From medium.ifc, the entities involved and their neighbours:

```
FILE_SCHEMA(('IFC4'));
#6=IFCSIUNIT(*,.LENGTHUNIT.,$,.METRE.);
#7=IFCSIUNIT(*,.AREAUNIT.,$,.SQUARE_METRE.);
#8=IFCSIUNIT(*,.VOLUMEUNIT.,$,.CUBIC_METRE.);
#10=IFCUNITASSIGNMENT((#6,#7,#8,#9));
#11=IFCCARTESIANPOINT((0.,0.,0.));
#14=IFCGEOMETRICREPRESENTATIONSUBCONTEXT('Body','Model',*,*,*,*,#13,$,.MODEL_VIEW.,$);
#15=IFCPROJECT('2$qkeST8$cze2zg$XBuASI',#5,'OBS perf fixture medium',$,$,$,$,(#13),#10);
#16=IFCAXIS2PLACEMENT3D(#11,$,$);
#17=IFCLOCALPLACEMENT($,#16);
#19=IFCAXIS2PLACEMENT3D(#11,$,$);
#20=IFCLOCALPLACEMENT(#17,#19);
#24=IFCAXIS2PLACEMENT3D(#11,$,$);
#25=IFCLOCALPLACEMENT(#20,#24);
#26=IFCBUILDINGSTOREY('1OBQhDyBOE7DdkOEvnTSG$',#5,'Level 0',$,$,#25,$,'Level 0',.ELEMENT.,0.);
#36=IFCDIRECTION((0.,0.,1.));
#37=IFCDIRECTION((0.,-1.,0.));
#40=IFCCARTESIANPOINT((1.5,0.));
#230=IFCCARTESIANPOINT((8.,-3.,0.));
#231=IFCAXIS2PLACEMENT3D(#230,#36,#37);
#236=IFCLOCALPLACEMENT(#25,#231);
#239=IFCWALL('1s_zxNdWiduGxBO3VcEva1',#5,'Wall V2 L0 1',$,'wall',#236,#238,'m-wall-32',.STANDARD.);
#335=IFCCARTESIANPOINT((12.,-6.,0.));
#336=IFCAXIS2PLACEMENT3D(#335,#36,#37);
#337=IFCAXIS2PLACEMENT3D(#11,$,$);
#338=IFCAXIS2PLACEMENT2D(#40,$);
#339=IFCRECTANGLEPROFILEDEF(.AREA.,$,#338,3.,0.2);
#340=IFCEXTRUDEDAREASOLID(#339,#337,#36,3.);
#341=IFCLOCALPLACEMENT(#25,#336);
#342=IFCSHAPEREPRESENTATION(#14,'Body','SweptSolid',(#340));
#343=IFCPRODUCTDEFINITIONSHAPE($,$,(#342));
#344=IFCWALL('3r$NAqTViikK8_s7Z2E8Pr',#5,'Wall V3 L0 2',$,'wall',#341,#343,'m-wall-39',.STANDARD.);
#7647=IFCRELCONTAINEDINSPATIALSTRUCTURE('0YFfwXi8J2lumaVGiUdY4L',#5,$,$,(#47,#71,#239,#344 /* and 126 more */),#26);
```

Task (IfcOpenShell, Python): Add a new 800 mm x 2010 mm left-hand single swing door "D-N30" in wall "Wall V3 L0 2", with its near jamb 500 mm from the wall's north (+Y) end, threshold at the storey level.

```python
import numpy as np
import ifcopenshell
import ifcopenshell.api.feature
import ifcopenshell.api.geometry
import ifcopenshell.api.root
import ifcopenshell.api.spatial
import ifcopenshell.geom
import ifcopenshell.util.element
import ifcopenshell.util.placement
import ifcopenshell.util.representation
import ifcopenshell.util.shape
import ifcopenshell.util.unit

model = ifcopenshell.open("medium.ifc")
unit_scale = ifcopenshell.util.unit.calculate_unit_scale(model)
settings = ifcopenshell.geom.settings()


def volume(element):
    """Net volume in cubic metres, openings subtracted."""
    shape = ifcopenshell.geom.create_shape(settings, element)
    return ifcopenshell.util.shape.get_volume(shape.geometry)


wall = model.by_guid("3r$NAqTViikK8_s7Z2E8Pr")
storey = ifcopenshell.util.element.get_container(wall, ifc_class="IfcBuildingStorey")
context = ifcopenshell.util.representation.get_context(model, "Model", "Body", "MODEL_VIEW")
before = volume(wall)

width, height, from_end, sill = 0.8, 2.01, 0.5, 0.0  # metres

# The wall runs along its own X axis, and the end named is its -X end.
wall_shape = ifcopenshell.geom.create_shape(settings, wall)
x, y, z = ifcopenshell.util.shape.get_vertices(wall_shape.geometry).T
start = x.min() + from_end
face, thickness = float(y.min()), float(y.max() - y.min())
wall_matrix = ifcopenshell.util.placement.get_local_placement(wall.ObjectPlacement)
level = ifcopenshell.util.placement.get_local_placement(storey.ObjectPlacement)[2, 3]


def in_wall(x, y):
    """Placement at x, y metres in the wall's axes, at sill height."""
    matrix = wall_matrix.copy()
    matrix[:, 3] = wall_matrix @ np.array([x / unit_scale, y / unit_scale, 0.0, 1.0])
    matrix[2, 3] = level + sill / unit_scale
    return matrix


# Opening: a box that overshoots both wall faces by 50 mm.
opening = ifcopenshell.api.root.create_entity(model, ifc_class="IfcOpeningElement", predefined_type="OPENING")
box = ifcopenshell.api.geometry.add_wall_representation(
    model, context=context, length=width, height=height, thickness=thickness + 0.1
)
ifcopenshell.api.geometry.assign_representation(model, product=opening, representation=box)
ifcopenshell.api.geometry.edit_object_placement(model, product=opening, matrix=in_wall(start, face - 0.05), is_si=False)
ifcopenshell.api.feature.add_feature(model, feature=opening, element=wall)

door = ifcopenshell.api.root.create_entity(model, ifc_class="IfcDoor", name="D-N30", predefined_type="DOOR")
door.OverallWidth, door.OverallHeight = width / unit_scale, height / unit_scale
door.OperationType = "SINGLE_SWING_LEFT"
body = ifcopenshell.api.geometry.add_door_representation(
    model,
    context=context,
    overall_width=door.OverallWidth,
    overall_height=door.OverallHeight,
    operation_type="SINGLE_SWING_LEFT",
    lining_properties={"LiningDepth": thickness / unit_scale, "ThresholdDepth": thickness / unit_scale},
)
ifcopenshell.api.geometry.assign_representation(model, product=door, representation=body)
ifcopenshell.api.spatial.assign_container(model, products=[door], relating_structure=storey)
ifcopenshell.api.feature.add_filling(model, opening=opening, element=door)

# The lining spans the wall, so the door starts at the wall face.
ifcopenshell.api.geometry.edit_object_placement(model, product=door, matrix=in_wall(start, face), is_si=False)

after = volume(wall)

print(f"wall volume {before:.3f} -> {after:.3f} m3")

model.write("medium_rev.ifc")
```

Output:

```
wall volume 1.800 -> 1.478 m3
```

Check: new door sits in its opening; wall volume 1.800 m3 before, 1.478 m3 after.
